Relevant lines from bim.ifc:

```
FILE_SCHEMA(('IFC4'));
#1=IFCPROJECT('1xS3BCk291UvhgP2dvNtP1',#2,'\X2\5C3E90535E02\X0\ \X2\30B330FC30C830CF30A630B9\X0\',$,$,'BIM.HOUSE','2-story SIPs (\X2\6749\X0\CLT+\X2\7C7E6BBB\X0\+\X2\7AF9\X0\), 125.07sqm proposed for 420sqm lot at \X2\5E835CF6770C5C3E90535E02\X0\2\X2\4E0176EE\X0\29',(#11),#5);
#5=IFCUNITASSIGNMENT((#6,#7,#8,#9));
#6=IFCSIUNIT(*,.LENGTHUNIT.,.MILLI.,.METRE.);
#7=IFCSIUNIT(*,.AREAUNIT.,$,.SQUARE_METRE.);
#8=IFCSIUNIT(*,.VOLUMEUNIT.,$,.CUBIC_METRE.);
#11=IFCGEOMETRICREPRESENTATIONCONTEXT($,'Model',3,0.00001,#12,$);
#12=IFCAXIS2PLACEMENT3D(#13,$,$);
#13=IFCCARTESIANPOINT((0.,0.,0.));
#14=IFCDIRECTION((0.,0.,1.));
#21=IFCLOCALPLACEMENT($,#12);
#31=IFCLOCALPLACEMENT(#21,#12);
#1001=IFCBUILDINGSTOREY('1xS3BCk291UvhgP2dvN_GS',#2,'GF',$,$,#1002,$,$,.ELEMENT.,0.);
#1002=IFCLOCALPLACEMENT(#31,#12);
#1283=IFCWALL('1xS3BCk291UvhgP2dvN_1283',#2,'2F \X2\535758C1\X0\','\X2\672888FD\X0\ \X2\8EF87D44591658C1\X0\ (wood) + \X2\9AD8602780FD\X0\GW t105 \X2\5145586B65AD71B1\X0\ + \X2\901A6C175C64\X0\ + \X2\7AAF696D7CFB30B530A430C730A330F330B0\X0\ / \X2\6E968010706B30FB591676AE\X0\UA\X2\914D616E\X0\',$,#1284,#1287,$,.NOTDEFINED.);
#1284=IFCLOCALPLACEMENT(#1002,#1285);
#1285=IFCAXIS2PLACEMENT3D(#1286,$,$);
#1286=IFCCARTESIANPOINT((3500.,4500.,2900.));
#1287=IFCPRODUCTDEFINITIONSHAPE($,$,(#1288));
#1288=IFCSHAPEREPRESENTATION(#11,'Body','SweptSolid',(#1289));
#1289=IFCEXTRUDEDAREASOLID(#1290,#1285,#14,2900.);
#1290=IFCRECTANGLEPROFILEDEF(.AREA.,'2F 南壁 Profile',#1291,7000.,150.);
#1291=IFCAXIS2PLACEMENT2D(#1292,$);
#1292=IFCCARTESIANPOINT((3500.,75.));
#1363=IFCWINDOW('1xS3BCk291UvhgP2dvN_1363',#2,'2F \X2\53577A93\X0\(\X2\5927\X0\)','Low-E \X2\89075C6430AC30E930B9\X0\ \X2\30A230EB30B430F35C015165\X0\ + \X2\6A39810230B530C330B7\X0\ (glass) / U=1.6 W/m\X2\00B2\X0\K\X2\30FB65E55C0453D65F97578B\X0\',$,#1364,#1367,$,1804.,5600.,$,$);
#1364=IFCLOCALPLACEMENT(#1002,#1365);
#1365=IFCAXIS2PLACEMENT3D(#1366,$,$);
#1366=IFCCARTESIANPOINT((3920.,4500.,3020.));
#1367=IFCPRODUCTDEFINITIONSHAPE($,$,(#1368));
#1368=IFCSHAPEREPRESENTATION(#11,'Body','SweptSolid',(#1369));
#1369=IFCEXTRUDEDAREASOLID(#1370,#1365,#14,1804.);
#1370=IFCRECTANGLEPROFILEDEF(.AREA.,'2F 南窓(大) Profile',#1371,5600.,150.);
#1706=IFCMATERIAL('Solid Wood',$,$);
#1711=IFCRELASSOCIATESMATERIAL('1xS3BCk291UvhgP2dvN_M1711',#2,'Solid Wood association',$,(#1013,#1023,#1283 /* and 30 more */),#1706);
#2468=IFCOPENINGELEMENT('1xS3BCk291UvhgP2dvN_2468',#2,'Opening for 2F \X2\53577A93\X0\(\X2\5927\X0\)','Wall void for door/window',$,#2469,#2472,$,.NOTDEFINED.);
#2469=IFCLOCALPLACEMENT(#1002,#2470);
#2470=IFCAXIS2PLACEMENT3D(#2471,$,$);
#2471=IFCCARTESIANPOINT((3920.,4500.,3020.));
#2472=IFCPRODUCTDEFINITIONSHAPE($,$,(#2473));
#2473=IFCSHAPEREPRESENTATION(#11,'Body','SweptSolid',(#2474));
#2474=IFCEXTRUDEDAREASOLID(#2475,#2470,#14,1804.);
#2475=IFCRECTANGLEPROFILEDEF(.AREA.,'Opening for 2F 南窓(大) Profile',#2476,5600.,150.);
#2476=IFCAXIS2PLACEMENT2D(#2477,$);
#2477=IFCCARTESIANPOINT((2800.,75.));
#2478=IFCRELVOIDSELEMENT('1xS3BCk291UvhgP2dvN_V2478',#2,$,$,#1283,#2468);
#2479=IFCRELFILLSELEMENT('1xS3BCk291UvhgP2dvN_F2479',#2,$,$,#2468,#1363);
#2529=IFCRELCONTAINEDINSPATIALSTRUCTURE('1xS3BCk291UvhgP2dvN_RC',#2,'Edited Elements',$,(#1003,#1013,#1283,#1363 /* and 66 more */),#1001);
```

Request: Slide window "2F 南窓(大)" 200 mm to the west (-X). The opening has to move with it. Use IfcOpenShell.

```python
import ifcopenshell
import ifcopenshell.api.geometry
import ifcopenshell.util.placement

model = ifcopenshell.open("bim.ifc")

window = model.by_guid("1xS3BCk291UvhgP2dvN_1363")
opening = window.FillsVoids[0].RelatingOpeningElement
wall = opening.VoidsElements[0].RelatingBuildingElement

wall_matrix = ifcopenshell.util.placement.get_local_placement(wall.ObjectPlacement)
shift = wall_matrix[:3, 0] * -200.0
before = ifcopenshell.util.placement.get_local_placement(window.ObjectPlacement)[:3, 3].copy()

# The window is not placed relative to its opening, so move both.
for product in (opening, window):
    matrix = ifcopenshell.util.placement.get_local_placement(product.ObjectPlacement)
    matrix[:3, 3] += shift
    ifcopenshell.api.geometry.edit_object_placement(model, product=product, matrix=matrix, is_si=False)

after = ifcopenshell.util.placement.get_local_placement(window.ObjectPlacement)[:3, 3]
print("window moved by", (after - before).round(3) + 0.0)

model.write("bim_rev.ifc")
```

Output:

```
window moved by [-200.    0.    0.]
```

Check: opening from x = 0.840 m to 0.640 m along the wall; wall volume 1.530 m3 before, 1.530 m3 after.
